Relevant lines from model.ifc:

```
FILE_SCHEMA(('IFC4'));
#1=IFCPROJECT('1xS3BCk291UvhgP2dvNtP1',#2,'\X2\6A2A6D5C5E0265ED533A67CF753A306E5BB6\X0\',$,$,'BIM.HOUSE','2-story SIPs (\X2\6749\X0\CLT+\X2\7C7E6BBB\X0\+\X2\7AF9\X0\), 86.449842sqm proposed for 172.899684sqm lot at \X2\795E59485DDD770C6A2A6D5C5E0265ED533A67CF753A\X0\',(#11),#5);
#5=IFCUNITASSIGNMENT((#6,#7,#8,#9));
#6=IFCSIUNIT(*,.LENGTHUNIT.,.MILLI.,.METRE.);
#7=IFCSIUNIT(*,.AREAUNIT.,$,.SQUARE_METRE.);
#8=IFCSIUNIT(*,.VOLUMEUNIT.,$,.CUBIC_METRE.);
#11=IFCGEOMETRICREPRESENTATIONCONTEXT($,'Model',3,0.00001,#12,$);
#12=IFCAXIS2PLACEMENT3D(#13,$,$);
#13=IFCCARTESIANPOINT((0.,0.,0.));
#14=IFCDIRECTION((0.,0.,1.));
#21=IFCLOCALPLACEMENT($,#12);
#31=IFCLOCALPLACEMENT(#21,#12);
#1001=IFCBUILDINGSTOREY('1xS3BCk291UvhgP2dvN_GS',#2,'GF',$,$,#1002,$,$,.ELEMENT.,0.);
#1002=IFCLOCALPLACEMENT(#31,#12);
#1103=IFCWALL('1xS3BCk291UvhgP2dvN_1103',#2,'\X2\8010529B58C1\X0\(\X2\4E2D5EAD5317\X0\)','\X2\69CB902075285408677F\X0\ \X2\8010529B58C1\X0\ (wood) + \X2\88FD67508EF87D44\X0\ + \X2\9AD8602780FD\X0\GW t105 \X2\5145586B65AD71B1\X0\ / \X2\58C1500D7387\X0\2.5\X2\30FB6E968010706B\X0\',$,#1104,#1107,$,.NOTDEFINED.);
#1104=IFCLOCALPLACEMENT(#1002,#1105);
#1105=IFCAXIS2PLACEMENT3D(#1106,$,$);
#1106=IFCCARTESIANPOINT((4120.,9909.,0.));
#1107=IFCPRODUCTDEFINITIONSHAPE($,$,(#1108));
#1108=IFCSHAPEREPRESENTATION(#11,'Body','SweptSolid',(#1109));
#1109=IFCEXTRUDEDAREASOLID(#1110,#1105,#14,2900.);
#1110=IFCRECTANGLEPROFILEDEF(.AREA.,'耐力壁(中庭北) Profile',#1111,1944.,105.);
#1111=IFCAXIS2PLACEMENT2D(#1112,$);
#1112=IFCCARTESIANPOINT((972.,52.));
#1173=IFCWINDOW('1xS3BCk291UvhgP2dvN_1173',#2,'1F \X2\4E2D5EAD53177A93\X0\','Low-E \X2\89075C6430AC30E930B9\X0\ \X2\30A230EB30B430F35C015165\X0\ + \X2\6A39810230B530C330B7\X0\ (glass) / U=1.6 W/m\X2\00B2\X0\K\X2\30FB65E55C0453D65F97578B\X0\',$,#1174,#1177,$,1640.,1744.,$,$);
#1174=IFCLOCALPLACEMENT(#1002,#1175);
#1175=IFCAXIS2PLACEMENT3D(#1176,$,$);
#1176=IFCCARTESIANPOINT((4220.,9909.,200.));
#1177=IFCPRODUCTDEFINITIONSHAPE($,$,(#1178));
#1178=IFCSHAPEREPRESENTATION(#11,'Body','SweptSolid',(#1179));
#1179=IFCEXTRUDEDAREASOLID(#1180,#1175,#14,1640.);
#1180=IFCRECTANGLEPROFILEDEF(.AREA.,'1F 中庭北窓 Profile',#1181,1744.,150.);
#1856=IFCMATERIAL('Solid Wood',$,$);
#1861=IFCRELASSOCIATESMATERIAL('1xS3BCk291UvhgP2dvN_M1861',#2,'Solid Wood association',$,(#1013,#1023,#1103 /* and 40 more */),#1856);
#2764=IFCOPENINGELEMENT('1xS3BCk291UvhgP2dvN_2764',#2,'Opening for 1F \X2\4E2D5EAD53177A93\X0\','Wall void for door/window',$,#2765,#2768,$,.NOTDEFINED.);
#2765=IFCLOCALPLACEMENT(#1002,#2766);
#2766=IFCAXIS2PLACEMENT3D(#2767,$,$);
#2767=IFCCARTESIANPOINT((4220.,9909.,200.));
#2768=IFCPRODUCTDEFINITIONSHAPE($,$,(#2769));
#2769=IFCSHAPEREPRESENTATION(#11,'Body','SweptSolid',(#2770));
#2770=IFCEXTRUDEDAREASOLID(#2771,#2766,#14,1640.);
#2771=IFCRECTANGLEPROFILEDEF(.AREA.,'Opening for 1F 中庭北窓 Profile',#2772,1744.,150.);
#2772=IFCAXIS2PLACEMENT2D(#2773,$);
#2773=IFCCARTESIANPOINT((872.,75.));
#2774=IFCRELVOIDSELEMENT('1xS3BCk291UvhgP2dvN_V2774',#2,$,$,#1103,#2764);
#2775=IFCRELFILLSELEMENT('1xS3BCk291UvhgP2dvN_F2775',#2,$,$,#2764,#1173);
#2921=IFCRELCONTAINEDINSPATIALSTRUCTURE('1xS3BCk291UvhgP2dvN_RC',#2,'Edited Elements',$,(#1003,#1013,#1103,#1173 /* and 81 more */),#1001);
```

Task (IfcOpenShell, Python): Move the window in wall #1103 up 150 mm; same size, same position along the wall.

```python
import numpy as np
import ifcopenshell
import ifcopenshell.api.geometry
import ifcopenshell.util.placement
import ifcopenshell.util.unit

model = ifcopenshell.open("model.ifc")
unit_scale = ifcopenshell.util.unit.calculate_unit_scale(model)

window = model.by_guid("1xS3BCk291UvhgP2dvN_1173")
opening = window.FillsVoids[0].RelatingOpeningElement
dz = 150.0

shift = np.array([0.0, 0.0, dz])
# The window is not placed relative to its opening, so move both.
for product in (opening, window):
    matrix = ifcopenshell.util.placement.get_local_placement(product.ObjectPlacement)
    matrix[:3, 3] += shift
    ifcopenshell.api.geometry.edit_object_placement(model, product=product, matrix=matrix, is_si=False)

print(f"moved by {dz * unit_scale:+.3f} m")

model.write("model-out.ifc")
```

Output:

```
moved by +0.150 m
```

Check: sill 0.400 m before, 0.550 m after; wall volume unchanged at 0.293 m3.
